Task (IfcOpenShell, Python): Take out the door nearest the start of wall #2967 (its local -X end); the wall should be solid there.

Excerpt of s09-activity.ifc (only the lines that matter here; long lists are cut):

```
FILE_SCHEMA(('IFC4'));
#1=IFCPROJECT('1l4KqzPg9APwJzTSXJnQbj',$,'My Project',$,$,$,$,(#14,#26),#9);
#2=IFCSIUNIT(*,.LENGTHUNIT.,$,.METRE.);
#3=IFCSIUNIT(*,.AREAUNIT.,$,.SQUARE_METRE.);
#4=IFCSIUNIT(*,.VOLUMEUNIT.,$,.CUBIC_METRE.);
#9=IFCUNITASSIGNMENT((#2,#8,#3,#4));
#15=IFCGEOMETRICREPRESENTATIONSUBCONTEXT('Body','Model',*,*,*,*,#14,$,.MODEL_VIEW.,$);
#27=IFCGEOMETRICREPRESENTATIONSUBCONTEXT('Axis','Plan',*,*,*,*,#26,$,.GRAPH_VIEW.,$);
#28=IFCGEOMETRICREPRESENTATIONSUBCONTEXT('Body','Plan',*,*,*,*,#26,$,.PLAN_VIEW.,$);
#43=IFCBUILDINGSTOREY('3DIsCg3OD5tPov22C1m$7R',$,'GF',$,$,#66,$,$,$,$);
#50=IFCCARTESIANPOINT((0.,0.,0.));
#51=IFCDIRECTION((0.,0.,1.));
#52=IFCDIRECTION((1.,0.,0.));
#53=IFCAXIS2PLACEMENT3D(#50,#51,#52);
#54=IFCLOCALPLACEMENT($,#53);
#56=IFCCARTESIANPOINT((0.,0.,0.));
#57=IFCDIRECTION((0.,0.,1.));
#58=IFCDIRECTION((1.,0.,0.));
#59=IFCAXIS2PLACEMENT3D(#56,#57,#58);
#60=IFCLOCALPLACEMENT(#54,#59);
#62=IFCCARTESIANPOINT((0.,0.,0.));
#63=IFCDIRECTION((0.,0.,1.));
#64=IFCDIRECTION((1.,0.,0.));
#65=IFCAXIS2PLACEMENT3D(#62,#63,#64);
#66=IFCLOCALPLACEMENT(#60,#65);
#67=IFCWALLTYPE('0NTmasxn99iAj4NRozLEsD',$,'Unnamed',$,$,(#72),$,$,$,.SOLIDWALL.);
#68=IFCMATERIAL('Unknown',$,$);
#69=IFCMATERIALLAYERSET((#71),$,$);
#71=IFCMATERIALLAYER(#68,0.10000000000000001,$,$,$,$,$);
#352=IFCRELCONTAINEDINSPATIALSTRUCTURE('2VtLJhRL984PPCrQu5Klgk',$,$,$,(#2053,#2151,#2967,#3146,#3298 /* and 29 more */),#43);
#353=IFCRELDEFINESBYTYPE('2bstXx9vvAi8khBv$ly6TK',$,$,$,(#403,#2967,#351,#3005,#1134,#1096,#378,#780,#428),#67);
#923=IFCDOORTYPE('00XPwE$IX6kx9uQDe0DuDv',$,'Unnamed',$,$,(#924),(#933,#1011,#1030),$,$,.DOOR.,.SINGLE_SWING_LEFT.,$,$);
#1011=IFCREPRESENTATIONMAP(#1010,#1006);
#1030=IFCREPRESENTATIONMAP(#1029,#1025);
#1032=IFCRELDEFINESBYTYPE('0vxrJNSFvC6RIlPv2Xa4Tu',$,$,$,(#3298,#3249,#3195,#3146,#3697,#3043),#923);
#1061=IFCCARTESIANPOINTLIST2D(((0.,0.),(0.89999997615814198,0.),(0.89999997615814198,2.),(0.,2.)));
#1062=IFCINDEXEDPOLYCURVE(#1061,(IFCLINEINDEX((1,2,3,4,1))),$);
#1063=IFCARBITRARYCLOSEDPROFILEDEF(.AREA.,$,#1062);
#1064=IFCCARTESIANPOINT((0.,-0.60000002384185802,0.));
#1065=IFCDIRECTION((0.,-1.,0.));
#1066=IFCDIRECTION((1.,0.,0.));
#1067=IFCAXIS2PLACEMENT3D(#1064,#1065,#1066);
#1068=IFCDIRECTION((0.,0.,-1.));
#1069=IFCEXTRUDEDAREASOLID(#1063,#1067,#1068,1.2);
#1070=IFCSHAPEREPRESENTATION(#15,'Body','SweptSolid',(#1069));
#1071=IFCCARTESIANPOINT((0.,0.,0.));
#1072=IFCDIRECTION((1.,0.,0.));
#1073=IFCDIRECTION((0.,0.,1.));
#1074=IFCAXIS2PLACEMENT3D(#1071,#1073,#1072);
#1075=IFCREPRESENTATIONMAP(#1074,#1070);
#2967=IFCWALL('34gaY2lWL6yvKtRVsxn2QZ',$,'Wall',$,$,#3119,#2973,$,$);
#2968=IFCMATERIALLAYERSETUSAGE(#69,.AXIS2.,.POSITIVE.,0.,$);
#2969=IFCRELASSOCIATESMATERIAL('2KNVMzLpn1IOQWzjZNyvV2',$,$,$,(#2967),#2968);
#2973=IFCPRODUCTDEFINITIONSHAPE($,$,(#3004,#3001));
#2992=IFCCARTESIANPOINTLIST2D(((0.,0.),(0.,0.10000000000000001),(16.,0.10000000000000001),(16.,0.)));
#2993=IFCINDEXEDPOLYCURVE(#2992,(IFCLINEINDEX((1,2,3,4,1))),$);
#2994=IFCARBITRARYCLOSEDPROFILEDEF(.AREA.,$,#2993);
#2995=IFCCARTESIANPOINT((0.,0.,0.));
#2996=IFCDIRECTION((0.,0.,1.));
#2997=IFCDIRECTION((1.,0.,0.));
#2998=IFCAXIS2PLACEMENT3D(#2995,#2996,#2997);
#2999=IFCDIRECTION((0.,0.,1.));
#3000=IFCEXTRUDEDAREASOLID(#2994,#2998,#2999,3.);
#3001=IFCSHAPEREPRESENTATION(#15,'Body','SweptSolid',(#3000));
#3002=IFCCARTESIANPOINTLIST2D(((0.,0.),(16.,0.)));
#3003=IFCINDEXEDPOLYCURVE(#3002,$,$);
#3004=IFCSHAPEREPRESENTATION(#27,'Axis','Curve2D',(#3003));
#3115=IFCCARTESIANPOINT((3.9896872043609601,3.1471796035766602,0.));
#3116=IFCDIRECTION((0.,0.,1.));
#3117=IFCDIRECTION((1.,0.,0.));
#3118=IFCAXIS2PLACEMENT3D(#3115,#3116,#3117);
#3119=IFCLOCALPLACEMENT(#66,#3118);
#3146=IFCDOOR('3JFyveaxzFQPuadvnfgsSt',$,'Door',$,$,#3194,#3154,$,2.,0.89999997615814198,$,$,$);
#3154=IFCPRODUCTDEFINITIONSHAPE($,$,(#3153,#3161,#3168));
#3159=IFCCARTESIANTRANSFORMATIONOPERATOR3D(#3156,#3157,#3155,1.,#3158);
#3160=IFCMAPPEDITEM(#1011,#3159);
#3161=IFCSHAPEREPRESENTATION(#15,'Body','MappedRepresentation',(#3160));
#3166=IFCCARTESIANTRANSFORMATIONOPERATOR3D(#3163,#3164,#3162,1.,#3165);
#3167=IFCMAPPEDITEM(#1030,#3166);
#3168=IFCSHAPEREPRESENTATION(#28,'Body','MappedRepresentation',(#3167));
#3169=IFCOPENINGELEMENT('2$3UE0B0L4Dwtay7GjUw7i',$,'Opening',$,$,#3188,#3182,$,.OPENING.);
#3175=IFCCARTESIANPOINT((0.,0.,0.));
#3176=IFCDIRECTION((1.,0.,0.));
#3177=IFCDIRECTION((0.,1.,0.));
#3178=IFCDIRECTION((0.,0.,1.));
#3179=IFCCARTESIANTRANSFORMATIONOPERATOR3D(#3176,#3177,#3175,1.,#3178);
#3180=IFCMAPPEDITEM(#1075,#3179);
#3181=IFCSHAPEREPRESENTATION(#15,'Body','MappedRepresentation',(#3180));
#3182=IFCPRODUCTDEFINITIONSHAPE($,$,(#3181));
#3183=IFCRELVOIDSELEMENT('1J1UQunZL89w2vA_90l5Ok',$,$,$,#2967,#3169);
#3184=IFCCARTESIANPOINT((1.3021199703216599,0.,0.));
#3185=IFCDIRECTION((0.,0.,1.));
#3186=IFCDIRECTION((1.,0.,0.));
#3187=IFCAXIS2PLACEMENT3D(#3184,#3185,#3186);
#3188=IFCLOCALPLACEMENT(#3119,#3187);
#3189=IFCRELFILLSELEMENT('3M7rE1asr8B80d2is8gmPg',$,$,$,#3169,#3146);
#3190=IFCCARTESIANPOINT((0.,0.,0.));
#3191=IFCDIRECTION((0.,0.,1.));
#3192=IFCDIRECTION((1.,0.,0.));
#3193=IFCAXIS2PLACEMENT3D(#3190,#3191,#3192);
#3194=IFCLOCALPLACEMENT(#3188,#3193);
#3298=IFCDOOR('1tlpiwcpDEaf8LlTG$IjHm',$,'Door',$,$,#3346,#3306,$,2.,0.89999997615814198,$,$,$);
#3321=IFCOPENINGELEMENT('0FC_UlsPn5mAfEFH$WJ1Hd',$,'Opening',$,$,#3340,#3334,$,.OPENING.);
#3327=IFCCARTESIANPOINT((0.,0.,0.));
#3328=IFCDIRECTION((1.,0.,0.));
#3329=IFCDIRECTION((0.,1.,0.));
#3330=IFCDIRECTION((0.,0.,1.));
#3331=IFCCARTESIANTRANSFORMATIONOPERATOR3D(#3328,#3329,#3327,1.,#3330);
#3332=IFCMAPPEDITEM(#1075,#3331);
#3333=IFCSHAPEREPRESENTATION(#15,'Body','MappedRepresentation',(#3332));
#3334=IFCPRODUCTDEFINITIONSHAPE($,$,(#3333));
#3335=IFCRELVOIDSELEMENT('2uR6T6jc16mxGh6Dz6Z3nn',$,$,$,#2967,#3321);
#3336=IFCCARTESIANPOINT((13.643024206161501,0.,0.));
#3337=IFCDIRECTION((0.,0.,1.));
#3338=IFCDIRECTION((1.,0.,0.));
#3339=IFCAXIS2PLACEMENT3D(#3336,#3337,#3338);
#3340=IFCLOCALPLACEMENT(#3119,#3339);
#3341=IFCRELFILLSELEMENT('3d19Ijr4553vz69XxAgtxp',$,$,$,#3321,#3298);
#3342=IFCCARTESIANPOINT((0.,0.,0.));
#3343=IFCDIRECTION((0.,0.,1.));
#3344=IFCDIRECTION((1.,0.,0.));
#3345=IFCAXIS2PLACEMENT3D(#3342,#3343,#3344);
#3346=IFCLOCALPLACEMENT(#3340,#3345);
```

```python
import ifcopenshell
import ifcopenshell.api.feature
import ifcopenshell.api.root
import ifcopenshell.geom
import ifcopenshell.util.shape

model = ifcopenshell.open("s09-activity.ifc")
settings = ifcopenshell.geom.settings()


def volume(element):
    """Net volume in cubic metres, openings subtracted."""
    shape = ifcopenshell.geom.create_shape(settings, element)
    return ifcopenshell.util.shape.get_volume(shape.geometry)


door = model.by_guid("3JFyveaxzFQPuadvnfgsSt")
opening = door.FillsVoids[0].RelatingOpeningElement
wall = opening.VoidsElements[0].RelatingBuildingElement
before = volume(wall)

ifcopenshell.api.root.remove_product(model, product=door)
ifcopenshell.api.feature.remove_feature(model, feature=opening)

after = volume(wall)

print(f"wall volume {before:.3f} -> {after:.3f} m3")

model.write("s09-activity_updated.ifc")
```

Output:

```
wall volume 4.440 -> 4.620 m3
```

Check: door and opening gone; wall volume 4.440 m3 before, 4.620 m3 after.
